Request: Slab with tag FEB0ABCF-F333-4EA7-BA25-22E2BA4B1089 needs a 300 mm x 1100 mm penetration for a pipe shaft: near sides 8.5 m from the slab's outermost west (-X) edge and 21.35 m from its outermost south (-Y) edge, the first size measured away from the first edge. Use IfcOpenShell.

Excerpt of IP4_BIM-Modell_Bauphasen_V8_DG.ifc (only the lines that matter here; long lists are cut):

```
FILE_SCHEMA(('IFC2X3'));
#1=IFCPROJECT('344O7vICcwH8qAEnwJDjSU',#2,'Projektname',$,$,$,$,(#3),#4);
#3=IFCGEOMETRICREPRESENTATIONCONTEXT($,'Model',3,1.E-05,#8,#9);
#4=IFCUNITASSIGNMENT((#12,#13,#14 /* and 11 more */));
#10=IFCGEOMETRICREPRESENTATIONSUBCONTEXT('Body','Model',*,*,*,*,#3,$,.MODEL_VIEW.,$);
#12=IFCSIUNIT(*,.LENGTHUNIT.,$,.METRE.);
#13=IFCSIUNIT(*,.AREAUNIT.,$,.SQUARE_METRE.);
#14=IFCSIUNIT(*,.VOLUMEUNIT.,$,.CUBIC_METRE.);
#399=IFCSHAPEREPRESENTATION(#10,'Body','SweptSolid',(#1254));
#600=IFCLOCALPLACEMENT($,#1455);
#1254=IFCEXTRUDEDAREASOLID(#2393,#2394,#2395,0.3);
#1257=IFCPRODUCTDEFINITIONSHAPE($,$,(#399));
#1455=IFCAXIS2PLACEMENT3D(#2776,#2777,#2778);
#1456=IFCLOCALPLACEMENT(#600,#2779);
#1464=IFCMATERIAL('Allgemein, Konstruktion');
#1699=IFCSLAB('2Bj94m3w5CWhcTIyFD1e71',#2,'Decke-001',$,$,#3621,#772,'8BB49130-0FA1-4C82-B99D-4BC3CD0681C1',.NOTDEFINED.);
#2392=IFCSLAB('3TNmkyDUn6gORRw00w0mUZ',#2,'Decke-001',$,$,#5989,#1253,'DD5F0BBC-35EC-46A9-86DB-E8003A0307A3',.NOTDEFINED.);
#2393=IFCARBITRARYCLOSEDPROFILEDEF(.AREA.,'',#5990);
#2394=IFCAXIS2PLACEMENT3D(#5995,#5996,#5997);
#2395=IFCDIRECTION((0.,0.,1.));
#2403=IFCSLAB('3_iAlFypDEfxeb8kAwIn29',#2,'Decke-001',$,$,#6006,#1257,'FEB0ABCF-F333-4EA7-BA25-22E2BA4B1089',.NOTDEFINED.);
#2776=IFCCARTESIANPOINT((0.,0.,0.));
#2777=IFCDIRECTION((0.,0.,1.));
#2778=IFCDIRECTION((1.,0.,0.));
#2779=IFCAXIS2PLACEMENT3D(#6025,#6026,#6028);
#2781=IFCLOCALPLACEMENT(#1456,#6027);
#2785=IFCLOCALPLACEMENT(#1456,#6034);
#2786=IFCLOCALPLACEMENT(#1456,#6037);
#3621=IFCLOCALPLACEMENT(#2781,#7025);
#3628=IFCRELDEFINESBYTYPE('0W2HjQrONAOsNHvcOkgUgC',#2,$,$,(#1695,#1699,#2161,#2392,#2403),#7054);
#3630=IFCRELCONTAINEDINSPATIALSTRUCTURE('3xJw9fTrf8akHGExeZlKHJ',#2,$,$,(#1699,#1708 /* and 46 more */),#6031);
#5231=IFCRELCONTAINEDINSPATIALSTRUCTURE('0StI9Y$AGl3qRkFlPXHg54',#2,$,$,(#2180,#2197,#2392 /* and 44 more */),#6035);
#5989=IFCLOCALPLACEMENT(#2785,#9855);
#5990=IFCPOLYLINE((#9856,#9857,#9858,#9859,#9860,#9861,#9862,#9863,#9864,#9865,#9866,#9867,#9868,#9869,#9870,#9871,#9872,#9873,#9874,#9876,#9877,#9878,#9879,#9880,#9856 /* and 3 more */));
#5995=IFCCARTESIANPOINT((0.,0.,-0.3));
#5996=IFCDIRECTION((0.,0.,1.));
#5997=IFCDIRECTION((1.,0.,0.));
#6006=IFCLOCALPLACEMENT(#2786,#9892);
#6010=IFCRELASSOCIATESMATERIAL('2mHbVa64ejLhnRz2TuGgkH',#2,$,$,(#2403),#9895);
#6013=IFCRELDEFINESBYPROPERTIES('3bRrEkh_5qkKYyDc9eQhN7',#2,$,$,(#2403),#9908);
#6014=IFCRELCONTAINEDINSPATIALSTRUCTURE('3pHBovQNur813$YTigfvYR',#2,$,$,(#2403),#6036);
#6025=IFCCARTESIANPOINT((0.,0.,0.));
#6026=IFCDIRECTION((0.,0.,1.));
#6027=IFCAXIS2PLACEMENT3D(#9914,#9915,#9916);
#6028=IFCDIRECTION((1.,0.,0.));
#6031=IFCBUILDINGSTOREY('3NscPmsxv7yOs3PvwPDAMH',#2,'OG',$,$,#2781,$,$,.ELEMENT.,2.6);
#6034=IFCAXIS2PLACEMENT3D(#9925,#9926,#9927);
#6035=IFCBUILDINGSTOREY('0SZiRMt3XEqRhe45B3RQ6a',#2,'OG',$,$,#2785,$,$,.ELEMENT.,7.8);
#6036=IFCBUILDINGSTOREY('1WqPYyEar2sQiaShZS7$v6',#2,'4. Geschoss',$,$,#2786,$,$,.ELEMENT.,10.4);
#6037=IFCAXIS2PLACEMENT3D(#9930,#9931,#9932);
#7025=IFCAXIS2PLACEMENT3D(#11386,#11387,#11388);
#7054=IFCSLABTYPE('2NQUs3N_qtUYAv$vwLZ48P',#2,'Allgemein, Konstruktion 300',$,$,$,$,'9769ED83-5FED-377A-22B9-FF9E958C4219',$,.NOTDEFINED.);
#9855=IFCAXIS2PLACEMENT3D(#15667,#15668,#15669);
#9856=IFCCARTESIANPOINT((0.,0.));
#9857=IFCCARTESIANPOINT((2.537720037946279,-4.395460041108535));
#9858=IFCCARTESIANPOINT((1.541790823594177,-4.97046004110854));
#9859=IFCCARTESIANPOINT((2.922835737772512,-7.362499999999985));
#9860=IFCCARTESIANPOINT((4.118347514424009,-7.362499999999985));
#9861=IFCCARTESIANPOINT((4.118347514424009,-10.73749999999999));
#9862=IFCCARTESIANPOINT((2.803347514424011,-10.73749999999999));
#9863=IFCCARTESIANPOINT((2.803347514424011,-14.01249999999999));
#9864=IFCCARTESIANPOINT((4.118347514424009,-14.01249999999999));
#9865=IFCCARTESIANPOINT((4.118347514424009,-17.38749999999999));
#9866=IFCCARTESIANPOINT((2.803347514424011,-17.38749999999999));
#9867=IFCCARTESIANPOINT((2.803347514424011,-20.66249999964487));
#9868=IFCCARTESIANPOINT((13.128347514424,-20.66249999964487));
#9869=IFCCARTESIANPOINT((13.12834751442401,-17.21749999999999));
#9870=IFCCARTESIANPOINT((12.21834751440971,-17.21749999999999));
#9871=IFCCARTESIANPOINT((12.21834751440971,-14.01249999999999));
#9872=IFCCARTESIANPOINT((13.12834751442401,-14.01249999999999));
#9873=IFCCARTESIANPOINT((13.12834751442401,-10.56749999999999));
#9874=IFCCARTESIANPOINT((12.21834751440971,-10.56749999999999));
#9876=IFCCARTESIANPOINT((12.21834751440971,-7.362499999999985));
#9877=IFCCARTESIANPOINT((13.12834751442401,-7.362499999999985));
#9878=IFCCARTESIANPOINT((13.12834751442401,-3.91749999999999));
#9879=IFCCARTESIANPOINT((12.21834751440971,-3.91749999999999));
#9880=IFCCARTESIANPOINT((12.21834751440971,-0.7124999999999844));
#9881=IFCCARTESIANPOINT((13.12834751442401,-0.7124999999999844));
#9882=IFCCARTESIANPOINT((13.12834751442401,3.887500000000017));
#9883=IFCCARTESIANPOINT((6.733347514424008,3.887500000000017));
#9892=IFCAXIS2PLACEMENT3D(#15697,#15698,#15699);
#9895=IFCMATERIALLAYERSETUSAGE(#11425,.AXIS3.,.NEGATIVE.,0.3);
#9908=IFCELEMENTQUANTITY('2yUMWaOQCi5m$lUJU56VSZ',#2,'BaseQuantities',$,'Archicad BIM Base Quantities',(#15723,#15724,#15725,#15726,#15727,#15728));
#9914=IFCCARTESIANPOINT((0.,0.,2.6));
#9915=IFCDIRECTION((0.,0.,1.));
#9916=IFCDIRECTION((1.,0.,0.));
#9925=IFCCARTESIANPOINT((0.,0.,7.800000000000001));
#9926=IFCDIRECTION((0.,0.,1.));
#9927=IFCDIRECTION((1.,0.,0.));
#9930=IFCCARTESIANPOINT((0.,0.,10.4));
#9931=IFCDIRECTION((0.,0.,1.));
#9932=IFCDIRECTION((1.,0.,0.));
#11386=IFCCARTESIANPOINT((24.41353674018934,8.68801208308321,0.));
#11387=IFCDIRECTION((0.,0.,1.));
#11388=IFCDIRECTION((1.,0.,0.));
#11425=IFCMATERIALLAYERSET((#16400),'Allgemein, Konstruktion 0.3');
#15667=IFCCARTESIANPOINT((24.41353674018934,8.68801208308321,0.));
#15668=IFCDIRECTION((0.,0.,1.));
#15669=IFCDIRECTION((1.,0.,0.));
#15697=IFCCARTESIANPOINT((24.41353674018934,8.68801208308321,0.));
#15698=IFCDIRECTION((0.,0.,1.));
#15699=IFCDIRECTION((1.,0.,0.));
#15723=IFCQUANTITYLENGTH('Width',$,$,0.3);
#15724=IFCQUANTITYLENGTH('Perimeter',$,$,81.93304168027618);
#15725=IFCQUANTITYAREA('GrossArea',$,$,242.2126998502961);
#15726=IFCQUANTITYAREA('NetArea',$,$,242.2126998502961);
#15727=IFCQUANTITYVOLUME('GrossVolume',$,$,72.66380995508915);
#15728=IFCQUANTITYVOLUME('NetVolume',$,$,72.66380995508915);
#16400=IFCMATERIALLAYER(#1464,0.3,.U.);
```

```python
import numpy as np
import ifcopenshell
import ifcopenshell.api.feature
import ifcopenshell.api.geometry
import ifcopenshell.api.pset
import ifcopenshell.api.root
import ifcopenshell.geom
import ifcopenshell.util.element
import ifcopenshell.util.placement
import ifcopenshell.util.representation
import ifcopenshell.util.shape
import ifcopenshell.util.unit

model = ifcopenshell.open("IP4_BIM-Modell_Bauphasen_V8_DG.ifc")
unit_scale = ifcopenshell.util.unit.calculate_unit_scale(model)
area_scale = ifcopenshell.util.unit.calculate_unit_scale(model, "AREAUNIT")
volume_scale = ifcopenshell.util.unit.calculate_unit_scale(model, "VOLUMEUNIT")
settings = ifcopenshell.geom.settings()


def volume(element):
    """Net volume in cubic metres, openings subtracted."""
    shape = ifcopenshell.geom.create_shape(settings, element)
    return ifcopenshell.util.shape.get_volume(shape.geometry)


slab = model.by_guid("3_iAlFypDEfxeb8kAwIn29")
before = volume(slab)

# Extent in the slab's own axes, in metres. The edges named are its -X and -Y sides.
slab_shape = ifcopenshell.geom.create_shape(settings, slab)
vertices = ifcopenshell.util.shape.get_vertices(slab_shape.geometry)
x_min, y_min, bottom = vertices.min(axis=0)
top = vertices[:, 2].max()

opening = ifcopenshell.api.root.create_entity(model, ifc_class="IfcOpeningElement", name="Pipe shaft opening")
context = ifcopenshell.util.representation.get_context(model, "Model", "Body", "MODEL_VIEW")
width, depth = 0.3, 1.1
outline = [(0.0, 0.0), (width, 0.0), (width, depth), (0.0, depth), (0.0, 0.0)]
# Overshoot both faces by 50 mm so the cut is clean.
shape = ifcopenshell.api.geometry.add_slab_representation(
    model, context=context, depth=top - bottom + 0.1, polyline=outline
)
ifcopenshell.api.geometry.assign_representation(model, product=opening, representation=shape)

matrix = ifcopenshell.util.placement.get_local_placement(slab.ObjectPlacement)
matrix[:, 3] = matrix @ np.append(np.array([x_min + 8.5, y_min + 21.35, bottom - 0.05]) / unit_scale, 1.0)
ifcopenshell.api.geometry.edit_object_placement(model, product=opening, matrix=matrix, is_si=False)
ifcopenshell.api.feature.add_feature(model, feature=opening, element=slab)

after = volume(slab)

# Update the slab's stored quantities.
qto = model.by_id(ifcopenshell.util.element.get_pset(slab, "BaseQuantities", should_inherit=False)["id"])
ifcopenshell.api.pset.edit_qto(model, qto=qto, properties={
    "NetArea": after / (top - bottom) / area_scale,
    "NetVolume": after / volume_scale,
})

print(f"slab volume {before:.3f} -> {after:.3f} m3")

model.write("IP4_BIM-Modell_Bauphasen_V8_DG_updated.ifc")
```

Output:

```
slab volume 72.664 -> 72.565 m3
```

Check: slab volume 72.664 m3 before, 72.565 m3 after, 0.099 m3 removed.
